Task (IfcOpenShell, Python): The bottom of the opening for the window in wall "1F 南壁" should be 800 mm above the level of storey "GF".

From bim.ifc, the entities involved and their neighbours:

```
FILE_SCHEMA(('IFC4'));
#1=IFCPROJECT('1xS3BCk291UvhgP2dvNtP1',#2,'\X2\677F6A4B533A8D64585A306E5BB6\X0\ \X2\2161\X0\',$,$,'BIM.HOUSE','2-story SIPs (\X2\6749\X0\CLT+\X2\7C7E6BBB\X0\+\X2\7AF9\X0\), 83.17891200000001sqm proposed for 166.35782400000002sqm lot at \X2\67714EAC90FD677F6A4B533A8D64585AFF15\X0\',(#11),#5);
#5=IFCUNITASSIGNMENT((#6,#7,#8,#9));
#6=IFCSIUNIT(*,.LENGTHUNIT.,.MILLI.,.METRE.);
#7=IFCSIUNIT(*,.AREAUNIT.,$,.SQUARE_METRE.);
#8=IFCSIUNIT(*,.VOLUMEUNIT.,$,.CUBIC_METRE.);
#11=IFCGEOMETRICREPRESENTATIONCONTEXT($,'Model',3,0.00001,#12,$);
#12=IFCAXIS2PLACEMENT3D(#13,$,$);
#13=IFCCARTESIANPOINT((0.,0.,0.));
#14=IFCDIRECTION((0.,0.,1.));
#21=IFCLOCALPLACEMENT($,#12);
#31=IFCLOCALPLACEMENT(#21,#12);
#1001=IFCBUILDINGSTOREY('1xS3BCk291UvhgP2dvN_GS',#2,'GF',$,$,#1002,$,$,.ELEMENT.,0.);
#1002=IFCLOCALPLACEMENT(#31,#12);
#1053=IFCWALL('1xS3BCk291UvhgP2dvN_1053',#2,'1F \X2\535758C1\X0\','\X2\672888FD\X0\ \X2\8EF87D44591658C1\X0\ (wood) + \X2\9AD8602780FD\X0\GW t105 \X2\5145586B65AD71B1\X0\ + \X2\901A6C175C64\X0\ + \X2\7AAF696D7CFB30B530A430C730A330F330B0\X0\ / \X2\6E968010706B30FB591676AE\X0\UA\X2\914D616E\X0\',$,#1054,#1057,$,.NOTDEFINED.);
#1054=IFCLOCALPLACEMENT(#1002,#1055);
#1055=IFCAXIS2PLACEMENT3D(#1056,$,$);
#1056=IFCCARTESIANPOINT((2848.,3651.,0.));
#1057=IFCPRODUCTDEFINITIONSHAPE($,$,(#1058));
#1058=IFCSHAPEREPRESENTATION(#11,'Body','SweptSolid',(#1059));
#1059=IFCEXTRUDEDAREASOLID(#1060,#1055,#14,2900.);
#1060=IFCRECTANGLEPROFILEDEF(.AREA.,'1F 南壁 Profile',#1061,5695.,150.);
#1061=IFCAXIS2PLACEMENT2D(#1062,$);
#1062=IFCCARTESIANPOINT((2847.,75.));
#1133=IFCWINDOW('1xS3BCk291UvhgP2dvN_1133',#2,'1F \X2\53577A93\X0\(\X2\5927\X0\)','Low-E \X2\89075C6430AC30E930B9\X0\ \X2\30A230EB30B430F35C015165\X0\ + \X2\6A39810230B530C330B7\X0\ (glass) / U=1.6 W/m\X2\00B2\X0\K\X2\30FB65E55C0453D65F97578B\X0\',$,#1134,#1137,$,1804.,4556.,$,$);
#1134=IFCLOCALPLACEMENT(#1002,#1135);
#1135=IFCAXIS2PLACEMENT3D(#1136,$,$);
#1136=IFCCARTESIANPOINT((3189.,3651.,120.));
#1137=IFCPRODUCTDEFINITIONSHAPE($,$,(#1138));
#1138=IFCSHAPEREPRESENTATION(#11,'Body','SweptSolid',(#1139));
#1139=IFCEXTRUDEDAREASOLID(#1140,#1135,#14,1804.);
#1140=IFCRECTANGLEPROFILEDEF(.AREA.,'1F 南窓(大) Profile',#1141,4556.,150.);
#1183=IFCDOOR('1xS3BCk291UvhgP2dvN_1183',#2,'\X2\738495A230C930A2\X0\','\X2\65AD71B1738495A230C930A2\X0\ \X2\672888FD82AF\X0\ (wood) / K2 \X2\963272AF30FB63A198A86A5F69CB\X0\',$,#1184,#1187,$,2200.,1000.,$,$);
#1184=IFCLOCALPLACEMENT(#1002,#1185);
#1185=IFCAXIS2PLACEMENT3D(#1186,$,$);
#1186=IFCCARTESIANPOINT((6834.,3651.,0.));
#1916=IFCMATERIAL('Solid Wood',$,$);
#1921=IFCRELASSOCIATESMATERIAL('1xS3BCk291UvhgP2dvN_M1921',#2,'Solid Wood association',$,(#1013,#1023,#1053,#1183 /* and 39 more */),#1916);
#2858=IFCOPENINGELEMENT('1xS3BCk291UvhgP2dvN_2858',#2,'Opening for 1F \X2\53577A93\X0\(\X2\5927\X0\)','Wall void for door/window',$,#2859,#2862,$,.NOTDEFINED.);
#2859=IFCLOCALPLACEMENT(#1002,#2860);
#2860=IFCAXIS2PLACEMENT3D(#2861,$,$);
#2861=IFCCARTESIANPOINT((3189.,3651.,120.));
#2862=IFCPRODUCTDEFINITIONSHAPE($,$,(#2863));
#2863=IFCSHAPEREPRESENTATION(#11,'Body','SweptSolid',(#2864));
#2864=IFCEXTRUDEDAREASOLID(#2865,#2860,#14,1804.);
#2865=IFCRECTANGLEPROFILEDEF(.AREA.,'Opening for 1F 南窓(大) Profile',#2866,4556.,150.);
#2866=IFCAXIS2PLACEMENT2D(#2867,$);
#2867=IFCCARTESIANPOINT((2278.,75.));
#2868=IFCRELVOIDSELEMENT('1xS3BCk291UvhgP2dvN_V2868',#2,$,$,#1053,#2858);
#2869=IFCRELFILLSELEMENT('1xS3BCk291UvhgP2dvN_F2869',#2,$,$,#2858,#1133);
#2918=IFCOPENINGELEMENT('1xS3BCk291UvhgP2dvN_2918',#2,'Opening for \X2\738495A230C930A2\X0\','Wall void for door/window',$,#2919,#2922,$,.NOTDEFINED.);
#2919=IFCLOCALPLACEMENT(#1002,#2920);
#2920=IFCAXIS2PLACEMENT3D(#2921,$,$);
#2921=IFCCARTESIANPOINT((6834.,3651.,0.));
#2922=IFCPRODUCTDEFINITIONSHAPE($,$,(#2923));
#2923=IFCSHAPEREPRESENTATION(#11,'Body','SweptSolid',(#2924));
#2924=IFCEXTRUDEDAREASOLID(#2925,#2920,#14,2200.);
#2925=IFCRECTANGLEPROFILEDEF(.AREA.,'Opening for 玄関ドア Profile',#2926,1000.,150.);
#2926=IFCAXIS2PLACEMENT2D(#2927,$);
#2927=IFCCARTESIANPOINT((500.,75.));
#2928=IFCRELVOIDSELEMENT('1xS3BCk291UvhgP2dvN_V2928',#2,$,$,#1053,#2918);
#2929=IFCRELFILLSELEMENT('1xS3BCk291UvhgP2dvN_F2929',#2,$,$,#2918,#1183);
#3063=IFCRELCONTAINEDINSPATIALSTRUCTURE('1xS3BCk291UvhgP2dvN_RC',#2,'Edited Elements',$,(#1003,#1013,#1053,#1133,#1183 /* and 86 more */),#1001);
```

```python
import numpy as np
import ifcopenshell
import ifcopenshell.api.geometry
import ifcopenshell.geom
import ifcopenshell.util.element
import ifcopenshell.util.placement
import ifcopenshell.util.shape
import ifcopenshell.util.unit

model = ifcopenshell.open("bim.ifc")
unit_scale = ifcopenshell.util.unit.calculate_unit_scale(model)

window = model.by_guid("1xS3BCk291UvhgP2dvN_1133")
opening = window.FillsVoids[0].RelatingOpeningElement
storey = ifcopenshell.util.element.get_container(window, ifc_class="IfcBuildingStorey")
level = ifcopenshell.util.placement.get_local_placement(storey.ObjectPlacement)[2, 3]

# The opening's origin need not be at the sill, so measure its lowest point.
shape = ifcopenshell.geom.create_shape(ifcopenshell.geom.settings(), opening)
bottom = ifcopenshell.util.shape.get_shape_bottom_elevation(shape, shape.geometry) / unit_scale
dz = level + 800.0 - bottom

shift = np.array([0.0, 0.0, dz])
# The window is not placed relative to its opening, so move both.
for product in (opening, window):
    matrix = ifcopenshell.util.placement.get_local_placement(product.ObjectPlacement)
    matrix[:3, 3] += shift
    ifcopenshell.api.geometry.edit_object_placement(model, product=product, matrix=matrix, is_si=False)

print(f"moved by {dz * unit_scale:+.3f} m")

model.write("bim_edited.ifc")
```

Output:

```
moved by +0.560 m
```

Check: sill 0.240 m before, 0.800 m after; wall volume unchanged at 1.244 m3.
